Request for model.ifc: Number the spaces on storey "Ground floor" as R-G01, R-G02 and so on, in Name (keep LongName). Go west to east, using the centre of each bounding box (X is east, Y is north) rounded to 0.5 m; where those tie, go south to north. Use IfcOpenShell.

First a look at what the model holds.

```python
import ifcopenshell
import ifcopenshell.util.element
import ifcopenshell.util.placement

model = ifcopenshell.open("model.ifc")
print(model.schema)
storey = next(s for s in model.by_type("IfcBuildingStorey") if s.Name == "Ground floor")
spaces = [e for e in ifcopenshell.util.element.get_decomposition(storey) if e.is_a("IfcSpace")]
for e in sorted(spaces, key=lambda e: e.id()):
    origin = ifcopenshell.util.placement.get_local_placement(e.ObjectPlacement)[:3, 3]
    print(e.id(), e.Name, e.LongName, origin.round(2) + 0.0, sep=" | ")
```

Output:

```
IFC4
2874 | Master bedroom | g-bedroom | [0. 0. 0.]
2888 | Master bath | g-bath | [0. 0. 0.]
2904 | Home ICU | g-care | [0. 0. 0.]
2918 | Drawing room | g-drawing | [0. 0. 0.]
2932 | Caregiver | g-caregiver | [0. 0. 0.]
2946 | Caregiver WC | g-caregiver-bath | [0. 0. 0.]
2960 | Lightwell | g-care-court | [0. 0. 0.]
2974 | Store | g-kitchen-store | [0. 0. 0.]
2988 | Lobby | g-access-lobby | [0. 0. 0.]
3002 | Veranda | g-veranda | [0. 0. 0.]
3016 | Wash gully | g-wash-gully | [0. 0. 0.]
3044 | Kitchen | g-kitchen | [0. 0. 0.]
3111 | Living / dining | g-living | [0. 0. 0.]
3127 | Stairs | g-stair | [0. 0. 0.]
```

```python
import ifcopenshell
import ifcopenshell.geom
import ifcopenshell.util.element
import ifcopenshell.util.shape

model = ifcopenshell.open("model.ifc")
settings = ifcopenshell.geom.settings()
settings.set("use-world-coords", True)


def centre(element):
    shape = ifcopenshell.geom.create_shape(settings, element)
    return ifcopenshell.util.shape.get_bbox_centroid(shape.geometry)


storey = next(s for s in model.by_type("IfcBuildingStorey") if s.Name == "Ground floor")
spaces = [e for e in ifcopenshell.util.element.get_decomposition(storey) if e.is_a("IfcSpace")]

# Insertion points can sit at a corner or the storey origin, so sort by the geometry (in metres).
centres = {e: centre(e) for e in spaces}
spaces.sort(key=lambda e: (round(centres[e][0] / 0.5), centres[e][1]))

for i, e in enumerate(spaces, start=1):
    number = f"R-G{i:02d}"
    e.Name = number
    print(e.id(), number)

model.write("model_v2.ifc")
```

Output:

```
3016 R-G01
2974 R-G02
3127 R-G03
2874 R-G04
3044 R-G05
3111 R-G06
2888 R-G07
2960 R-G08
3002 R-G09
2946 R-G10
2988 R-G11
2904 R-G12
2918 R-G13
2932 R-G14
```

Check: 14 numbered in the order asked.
